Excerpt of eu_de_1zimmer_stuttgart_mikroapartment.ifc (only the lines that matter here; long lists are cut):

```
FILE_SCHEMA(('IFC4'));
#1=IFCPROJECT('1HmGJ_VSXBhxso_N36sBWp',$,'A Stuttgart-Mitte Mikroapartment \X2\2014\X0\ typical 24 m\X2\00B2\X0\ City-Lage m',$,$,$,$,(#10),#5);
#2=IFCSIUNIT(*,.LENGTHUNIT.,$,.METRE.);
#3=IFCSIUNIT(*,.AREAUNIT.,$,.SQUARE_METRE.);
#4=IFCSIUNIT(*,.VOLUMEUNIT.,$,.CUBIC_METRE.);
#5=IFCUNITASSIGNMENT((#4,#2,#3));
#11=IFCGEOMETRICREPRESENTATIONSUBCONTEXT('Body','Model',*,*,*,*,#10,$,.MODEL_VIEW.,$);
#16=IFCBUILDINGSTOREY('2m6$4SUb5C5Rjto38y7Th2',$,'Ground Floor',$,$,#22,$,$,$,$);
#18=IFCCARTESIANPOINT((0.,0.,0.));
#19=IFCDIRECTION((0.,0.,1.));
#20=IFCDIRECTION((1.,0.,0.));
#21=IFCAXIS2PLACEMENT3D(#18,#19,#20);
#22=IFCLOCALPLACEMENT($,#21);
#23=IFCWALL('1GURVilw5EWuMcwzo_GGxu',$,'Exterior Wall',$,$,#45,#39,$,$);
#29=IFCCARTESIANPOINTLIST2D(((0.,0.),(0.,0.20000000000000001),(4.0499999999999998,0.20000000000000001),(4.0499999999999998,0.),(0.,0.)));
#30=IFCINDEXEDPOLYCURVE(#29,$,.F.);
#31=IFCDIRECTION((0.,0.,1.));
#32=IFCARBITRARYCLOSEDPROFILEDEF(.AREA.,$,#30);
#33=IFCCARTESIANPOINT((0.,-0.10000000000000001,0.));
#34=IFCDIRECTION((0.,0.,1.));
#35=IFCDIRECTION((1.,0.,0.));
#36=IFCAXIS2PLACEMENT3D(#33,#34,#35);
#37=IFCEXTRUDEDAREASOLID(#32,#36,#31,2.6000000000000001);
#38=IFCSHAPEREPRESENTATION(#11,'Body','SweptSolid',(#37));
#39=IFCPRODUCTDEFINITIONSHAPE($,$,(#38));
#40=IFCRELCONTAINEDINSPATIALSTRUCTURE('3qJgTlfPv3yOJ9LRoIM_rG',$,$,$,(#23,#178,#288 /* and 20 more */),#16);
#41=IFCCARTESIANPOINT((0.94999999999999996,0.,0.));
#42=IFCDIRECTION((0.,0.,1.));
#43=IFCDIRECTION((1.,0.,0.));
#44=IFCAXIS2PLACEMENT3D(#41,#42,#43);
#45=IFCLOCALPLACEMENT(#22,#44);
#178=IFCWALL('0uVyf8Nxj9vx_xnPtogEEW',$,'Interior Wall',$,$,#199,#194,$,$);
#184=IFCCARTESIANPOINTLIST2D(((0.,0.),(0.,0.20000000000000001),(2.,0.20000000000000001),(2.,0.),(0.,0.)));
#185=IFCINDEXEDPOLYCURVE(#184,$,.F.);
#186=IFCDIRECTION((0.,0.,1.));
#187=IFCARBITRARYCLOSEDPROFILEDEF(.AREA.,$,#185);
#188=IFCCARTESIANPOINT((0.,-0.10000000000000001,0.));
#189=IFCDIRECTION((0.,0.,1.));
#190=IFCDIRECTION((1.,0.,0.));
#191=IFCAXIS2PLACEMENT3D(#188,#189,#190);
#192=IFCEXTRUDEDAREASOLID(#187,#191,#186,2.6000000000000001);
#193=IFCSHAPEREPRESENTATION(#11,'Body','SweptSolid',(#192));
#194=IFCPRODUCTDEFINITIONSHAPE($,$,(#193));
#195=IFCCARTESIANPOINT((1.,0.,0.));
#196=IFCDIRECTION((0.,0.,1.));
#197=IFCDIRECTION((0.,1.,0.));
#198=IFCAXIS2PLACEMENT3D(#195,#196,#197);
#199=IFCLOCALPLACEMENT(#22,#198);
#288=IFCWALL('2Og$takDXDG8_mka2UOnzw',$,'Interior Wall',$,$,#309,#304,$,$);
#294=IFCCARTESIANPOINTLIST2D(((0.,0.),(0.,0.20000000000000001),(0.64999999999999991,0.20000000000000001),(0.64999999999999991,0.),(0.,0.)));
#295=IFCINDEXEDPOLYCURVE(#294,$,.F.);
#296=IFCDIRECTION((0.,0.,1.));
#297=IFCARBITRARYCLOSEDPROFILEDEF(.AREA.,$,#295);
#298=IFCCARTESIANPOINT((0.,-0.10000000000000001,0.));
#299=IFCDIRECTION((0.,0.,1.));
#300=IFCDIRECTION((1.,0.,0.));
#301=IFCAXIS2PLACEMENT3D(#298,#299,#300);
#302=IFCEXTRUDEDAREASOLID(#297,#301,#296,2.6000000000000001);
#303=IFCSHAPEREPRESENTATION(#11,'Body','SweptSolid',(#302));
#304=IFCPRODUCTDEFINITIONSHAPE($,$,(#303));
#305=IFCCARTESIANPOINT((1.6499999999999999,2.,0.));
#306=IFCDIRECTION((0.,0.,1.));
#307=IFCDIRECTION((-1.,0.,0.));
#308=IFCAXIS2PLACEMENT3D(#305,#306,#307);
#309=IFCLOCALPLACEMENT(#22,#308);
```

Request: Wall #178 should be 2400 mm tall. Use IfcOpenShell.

```python
import ifcopenshell
import ifcopenshell.geom
import ifcopenshell.util.representation
import ifcopenshell.util.shape

model = ifcopenshell.open("eu_de_1zimmer_stuttgart_mikroapartment.ifc")
settings = ifcopenshell.geom.settings()


def volume(element):
    """Net volume in cubic metres, openings subtracted."""
    shape = ifcopenshell.geom.create_shape(settings, element)
    return ifcopenshell.util.shape.get_volume(shape.geometry)


wall = model.by_guid("0uVyf8Nxj9vx_xnPtogEEW")
before = volume(wall)

body = ifcopenshell.util.representation.get_representation(wall, "Model", "Body")
solid = body.Items[0]
old_height = solid.Depth
solid.Depth = 2.4
after = volume(wall)

print(f"height {old_height:g} -> {solid.Depth:g}, volume {before:.3f} -> {after:.3f} m3")

model.write("eu_de_1zimmer_stuttgart_mikroapartment_rev.ifc")
```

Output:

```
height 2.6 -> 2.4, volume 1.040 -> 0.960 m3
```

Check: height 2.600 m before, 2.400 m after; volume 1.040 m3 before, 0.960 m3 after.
